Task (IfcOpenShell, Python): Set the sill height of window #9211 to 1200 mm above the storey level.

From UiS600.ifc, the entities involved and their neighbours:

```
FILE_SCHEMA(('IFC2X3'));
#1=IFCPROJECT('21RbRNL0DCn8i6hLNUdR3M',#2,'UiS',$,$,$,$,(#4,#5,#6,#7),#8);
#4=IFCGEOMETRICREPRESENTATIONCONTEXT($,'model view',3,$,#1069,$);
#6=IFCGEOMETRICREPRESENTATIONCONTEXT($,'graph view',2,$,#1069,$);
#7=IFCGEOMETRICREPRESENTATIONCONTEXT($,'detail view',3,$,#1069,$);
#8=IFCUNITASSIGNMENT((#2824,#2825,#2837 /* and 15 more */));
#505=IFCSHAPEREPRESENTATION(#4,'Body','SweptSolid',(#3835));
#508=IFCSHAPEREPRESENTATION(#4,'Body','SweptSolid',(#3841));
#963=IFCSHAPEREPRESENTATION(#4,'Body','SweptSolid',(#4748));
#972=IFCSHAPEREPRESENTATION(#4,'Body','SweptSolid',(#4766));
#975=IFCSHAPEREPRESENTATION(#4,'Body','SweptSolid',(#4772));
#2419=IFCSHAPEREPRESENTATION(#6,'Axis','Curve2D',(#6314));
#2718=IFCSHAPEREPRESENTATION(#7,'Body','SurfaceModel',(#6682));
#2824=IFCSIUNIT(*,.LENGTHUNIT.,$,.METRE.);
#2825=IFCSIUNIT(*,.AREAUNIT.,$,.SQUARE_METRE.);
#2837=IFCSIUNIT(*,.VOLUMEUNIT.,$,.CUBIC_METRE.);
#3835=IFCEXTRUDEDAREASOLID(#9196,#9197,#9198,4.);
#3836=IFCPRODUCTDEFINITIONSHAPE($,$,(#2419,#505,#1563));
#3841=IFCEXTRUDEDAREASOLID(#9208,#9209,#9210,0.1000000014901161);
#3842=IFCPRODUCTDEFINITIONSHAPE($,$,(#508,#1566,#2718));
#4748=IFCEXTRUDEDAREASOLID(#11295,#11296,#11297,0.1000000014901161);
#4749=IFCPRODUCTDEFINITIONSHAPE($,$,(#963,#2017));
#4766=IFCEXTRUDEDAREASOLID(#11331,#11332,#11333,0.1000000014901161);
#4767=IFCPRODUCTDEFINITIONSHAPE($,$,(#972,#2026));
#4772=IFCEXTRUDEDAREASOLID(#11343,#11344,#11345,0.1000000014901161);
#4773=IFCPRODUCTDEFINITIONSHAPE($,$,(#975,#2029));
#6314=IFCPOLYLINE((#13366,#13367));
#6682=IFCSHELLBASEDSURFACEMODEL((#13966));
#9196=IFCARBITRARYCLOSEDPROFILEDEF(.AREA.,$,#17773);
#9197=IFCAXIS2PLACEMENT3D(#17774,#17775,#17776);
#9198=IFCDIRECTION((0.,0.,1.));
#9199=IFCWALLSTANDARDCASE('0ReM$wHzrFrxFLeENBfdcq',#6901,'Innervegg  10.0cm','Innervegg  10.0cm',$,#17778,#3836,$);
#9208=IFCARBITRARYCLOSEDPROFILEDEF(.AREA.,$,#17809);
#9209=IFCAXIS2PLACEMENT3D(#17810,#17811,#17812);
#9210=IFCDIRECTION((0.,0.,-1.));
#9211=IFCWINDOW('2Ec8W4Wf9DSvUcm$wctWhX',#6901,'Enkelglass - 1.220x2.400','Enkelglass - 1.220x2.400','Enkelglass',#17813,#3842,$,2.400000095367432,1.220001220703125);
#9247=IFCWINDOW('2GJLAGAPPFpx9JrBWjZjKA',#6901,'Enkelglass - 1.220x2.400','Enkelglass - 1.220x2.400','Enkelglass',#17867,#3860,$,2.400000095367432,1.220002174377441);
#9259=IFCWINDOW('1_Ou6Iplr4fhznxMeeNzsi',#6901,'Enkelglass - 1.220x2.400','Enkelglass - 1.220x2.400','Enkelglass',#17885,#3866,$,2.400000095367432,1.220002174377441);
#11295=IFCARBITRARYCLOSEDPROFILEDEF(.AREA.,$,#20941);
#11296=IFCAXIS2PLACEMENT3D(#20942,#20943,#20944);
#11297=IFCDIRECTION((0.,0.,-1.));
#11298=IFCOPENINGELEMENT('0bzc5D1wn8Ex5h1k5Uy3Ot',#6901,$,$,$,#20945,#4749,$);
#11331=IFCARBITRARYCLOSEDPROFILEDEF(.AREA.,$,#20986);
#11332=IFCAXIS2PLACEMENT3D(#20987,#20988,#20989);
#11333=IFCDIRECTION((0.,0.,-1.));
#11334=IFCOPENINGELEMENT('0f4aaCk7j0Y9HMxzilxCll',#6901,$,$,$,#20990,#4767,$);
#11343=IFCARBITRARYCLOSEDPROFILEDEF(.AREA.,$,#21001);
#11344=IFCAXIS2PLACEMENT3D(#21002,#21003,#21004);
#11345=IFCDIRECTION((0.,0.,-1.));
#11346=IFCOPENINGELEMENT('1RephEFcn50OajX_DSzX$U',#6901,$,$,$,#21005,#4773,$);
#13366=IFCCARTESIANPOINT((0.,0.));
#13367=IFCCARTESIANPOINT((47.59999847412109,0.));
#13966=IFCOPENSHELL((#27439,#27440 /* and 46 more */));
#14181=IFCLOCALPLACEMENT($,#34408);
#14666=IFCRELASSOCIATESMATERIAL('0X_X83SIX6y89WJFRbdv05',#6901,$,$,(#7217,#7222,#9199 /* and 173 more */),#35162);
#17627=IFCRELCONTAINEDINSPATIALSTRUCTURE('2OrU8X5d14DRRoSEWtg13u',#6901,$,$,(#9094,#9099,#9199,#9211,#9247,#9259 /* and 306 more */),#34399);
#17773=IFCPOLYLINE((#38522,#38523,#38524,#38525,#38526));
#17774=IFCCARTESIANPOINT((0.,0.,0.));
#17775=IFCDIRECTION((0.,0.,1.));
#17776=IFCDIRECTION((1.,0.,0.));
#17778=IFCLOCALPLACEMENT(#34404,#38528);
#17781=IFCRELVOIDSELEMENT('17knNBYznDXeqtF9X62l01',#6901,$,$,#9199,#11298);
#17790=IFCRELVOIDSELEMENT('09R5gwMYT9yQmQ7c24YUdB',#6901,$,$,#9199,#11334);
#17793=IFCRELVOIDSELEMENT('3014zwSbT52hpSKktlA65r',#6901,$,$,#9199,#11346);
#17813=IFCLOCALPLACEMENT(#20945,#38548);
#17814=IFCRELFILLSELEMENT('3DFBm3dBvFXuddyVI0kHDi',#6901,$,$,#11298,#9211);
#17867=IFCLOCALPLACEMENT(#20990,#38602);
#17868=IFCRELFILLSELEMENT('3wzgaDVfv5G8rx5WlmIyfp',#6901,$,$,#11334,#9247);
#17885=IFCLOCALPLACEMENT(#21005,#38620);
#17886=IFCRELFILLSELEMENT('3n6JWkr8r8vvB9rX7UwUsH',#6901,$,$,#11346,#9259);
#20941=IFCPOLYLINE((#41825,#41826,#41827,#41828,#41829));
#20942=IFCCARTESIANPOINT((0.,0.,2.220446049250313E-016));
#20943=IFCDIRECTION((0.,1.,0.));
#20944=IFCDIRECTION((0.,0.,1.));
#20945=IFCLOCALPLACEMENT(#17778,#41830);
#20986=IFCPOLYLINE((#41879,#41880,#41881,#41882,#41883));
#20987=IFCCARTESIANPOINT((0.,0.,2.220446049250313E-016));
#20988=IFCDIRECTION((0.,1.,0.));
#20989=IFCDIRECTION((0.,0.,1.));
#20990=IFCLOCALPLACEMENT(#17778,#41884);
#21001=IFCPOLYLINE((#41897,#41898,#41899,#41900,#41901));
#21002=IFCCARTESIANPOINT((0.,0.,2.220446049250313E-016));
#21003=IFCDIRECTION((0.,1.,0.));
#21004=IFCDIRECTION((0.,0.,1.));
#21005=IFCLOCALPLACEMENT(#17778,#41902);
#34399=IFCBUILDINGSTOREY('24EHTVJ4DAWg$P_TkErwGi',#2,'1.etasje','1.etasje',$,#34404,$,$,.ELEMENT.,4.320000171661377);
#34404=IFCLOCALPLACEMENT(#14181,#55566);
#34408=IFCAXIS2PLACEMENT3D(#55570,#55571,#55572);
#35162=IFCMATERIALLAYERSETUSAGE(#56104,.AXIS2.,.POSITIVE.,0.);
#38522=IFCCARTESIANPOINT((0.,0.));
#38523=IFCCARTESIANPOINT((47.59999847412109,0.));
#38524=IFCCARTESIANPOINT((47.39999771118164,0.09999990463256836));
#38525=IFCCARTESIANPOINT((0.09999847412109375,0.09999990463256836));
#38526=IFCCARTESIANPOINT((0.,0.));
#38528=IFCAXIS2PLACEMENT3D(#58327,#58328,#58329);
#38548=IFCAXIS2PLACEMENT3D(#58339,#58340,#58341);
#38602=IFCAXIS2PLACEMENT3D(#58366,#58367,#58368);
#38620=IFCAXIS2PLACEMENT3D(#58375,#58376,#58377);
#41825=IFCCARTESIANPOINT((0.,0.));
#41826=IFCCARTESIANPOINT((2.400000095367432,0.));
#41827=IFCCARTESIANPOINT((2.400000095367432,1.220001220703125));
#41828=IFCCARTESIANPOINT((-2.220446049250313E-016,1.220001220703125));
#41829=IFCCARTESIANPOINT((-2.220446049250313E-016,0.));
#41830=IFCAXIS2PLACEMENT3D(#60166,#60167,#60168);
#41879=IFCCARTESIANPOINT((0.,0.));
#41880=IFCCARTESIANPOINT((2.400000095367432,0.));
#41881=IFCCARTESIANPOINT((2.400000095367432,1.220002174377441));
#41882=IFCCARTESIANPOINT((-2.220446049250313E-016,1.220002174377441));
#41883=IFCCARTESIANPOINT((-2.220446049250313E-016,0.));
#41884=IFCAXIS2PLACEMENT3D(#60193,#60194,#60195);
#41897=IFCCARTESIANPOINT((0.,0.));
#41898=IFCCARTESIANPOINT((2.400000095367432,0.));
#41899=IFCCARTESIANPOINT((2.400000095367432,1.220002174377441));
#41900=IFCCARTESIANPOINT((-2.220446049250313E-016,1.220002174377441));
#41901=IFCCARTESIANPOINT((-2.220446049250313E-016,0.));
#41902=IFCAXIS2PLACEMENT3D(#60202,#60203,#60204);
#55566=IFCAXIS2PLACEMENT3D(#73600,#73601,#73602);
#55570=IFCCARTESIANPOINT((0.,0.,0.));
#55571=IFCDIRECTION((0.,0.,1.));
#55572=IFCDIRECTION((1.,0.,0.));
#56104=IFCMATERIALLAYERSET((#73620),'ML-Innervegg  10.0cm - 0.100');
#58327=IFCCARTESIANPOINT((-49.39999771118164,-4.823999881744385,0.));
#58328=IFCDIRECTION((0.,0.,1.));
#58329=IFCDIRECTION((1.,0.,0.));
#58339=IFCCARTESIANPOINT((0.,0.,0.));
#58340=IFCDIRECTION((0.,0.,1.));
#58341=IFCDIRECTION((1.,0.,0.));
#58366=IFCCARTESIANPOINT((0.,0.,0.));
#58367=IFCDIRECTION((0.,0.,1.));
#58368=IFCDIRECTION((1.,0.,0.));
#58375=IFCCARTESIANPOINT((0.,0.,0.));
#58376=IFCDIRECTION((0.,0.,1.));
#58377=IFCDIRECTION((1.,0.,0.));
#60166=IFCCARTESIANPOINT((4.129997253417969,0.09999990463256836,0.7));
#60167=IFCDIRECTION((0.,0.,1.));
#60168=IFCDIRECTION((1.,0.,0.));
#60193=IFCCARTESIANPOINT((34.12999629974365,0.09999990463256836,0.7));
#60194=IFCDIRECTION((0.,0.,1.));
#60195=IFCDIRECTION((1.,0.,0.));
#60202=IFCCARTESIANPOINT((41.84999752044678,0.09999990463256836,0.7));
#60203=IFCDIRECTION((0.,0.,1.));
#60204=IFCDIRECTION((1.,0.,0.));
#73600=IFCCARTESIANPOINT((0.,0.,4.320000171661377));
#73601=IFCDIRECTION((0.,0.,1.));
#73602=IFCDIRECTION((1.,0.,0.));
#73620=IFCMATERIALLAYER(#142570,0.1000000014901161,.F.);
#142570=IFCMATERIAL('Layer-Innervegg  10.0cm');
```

```python
import numpy as np
import ifcopenshell
import ifcopenshell.api.geometry
import ifcopenshell.geom
import ifcopenshell.util.element
import ifcopenshell.util.placement
import ifcopenshell.util.shape
import ifcopenshell.util.unit

model = ifcopenshell.open("UiS600.ifc")
unit_scale = ifcopenshell.util.unit.calculate_unit_scale(model)

window = model.by_id(9211)
opening = window.FillsVoids[0].RelatingOpeningElement
storey = ifcopenshell.util.element.get_container(window, ifc_class="IfcBuildingStorey")
level = ifcopenshell.util.placement.get_local_placement(storey.ObjectPlacement)[2, 3]

# The opening's origin need not be at the sill, so measure its lowest point.
shape = ifcopenshell.geom.create_shape(ifcopenshell.geom.settings(), opening)
bottom = ifcopenshell.util.shape.get_shape_bottom_elevation(shape, shape.geometry) / unit_scale
dz = level + 1.2 / unit_scale - bottom

shift = np.array([0.0, 0.0, dz])
# The window is placed relative to its opening, so it follows when the opening moves.
matrix = ifcopenshell.util.placement.get_local_placement(opening.ObjectPlacement)
matrix[:3, 3] += shift
ifcopenshell.api.geometry.edit_object_placement(
    model, product=opening, matrix=matrix, is_si=False, should_transform_children=True
)

print(f"moved by {dz * unit_scale:+.3f} m")

model.write("UiS600_rev.ifc")
```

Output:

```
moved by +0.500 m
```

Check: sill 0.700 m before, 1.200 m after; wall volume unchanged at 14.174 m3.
